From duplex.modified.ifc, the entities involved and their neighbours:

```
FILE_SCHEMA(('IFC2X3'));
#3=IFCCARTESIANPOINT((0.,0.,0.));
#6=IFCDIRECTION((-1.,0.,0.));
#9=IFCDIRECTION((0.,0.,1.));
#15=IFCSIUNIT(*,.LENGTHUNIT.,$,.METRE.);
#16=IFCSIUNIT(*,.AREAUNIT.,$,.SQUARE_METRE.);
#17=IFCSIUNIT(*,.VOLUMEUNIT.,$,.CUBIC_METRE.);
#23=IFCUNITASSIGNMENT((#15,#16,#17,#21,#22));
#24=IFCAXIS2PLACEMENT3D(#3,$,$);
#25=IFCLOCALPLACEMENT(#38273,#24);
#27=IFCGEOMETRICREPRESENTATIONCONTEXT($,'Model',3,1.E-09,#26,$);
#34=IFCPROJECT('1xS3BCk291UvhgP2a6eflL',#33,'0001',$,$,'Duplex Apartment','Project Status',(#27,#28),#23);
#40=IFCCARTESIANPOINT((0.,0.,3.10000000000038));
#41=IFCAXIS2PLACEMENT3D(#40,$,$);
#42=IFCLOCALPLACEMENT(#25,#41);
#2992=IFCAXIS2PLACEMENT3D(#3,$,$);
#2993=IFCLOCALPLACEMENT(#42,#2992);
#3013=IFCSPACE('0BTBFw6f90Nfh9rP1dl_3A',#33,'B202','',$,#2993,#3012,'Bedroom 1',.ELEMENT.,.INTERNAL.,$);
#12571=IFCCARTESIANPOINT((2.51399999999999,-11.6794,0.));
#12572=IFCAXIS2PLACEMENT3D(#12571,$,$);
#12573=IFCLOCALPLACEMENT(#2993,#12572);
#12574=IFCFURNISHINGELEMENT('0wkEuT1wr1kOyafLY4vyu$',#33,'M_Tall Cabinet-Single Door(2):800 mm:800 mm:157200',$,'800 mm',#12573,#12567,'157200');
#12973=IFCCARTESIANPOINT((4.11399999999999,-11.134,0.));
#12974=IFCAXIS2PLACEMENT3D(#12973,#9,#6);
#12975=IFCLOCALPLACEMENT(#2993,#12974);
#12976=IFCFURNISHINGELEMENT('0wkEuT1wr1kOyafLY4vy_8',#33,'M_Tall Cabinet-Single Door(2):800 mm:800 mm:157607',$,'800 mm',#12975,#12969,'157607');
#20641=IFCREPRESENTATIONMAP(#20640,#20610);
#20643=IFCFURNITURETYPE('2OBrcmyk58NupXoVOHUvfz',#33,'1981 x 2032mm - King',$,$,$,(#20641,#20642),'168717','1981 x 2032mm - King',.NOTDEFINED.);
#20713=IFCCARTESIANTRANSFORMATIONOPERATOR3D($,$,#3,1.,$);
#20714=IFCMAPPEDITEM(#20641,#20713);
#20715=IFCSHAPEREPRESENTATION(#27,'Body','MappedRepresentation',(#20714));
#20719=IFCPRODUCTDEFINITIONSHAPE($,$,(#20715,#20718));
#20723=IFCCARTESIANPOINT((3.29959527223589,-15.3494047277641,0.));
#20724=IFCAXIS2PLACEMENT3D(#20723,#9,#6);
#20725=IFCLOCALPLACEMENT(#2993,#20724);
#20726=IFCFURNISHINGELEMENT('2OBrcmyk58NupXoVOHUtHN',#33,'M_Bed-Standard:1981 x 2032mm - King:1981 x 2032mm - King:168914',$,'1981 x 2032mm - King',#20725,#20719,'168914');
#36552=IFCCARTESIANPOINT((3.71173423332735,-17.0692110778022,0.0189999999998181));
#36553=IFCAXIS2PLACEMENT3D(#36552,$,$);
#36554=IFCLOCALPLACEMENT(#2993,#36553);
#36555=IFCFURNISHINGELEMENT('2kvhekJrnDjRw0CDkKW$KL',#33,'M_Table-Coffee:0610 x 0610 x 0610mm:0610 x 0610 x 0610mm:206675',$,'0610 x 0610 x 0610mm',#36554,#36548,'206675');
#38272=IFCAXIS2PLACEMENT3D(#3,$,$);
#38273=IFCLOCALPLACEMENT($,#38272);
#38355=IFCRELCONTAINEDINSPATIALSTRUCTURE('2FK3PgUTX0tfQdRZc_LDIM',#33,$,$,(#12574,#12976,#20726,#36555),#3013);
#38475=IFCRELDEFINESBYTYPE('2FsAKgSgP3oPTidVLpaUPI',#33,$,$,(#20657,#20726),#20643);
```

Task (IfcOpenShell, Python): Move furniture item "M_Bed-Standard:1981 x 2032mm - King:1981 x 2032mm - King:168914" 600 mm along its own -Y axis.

```python
import ifcopenshell
import ifcopenshell.api.geometry
import ifcopenshell.util.placement
import ifcopenshell.util.unit

model = ifcopenshell.open("duplex.modified.ifc")
unit_scale = ifcopenshell.util.unit.calculate_unit_scale(model)

item = model.by_guid("2OBrcmyk58NupXoVOHUtHN")
matrix = ifcopenshell.util.placement.get_local_placement(item.ObjectPlacement)
matrix[:3, 3] -= matrix[:3, 1] * 0.6 / unit_scale
ifcopenshell.api.geometry.edit_object_placement(model, product=item, matrix=matrix, is_si=False)

print(ifcopenshell.util.placement.get_local_placement(item.ObjectPlacement).round(3) + 0.0)

model.write("duplex.modified-out.ifc")
```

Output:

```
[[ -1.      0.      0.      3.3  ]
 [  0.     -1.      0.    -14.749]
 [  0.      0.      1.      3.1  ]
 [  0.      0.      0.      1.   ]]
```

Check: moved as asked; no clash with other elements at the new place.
